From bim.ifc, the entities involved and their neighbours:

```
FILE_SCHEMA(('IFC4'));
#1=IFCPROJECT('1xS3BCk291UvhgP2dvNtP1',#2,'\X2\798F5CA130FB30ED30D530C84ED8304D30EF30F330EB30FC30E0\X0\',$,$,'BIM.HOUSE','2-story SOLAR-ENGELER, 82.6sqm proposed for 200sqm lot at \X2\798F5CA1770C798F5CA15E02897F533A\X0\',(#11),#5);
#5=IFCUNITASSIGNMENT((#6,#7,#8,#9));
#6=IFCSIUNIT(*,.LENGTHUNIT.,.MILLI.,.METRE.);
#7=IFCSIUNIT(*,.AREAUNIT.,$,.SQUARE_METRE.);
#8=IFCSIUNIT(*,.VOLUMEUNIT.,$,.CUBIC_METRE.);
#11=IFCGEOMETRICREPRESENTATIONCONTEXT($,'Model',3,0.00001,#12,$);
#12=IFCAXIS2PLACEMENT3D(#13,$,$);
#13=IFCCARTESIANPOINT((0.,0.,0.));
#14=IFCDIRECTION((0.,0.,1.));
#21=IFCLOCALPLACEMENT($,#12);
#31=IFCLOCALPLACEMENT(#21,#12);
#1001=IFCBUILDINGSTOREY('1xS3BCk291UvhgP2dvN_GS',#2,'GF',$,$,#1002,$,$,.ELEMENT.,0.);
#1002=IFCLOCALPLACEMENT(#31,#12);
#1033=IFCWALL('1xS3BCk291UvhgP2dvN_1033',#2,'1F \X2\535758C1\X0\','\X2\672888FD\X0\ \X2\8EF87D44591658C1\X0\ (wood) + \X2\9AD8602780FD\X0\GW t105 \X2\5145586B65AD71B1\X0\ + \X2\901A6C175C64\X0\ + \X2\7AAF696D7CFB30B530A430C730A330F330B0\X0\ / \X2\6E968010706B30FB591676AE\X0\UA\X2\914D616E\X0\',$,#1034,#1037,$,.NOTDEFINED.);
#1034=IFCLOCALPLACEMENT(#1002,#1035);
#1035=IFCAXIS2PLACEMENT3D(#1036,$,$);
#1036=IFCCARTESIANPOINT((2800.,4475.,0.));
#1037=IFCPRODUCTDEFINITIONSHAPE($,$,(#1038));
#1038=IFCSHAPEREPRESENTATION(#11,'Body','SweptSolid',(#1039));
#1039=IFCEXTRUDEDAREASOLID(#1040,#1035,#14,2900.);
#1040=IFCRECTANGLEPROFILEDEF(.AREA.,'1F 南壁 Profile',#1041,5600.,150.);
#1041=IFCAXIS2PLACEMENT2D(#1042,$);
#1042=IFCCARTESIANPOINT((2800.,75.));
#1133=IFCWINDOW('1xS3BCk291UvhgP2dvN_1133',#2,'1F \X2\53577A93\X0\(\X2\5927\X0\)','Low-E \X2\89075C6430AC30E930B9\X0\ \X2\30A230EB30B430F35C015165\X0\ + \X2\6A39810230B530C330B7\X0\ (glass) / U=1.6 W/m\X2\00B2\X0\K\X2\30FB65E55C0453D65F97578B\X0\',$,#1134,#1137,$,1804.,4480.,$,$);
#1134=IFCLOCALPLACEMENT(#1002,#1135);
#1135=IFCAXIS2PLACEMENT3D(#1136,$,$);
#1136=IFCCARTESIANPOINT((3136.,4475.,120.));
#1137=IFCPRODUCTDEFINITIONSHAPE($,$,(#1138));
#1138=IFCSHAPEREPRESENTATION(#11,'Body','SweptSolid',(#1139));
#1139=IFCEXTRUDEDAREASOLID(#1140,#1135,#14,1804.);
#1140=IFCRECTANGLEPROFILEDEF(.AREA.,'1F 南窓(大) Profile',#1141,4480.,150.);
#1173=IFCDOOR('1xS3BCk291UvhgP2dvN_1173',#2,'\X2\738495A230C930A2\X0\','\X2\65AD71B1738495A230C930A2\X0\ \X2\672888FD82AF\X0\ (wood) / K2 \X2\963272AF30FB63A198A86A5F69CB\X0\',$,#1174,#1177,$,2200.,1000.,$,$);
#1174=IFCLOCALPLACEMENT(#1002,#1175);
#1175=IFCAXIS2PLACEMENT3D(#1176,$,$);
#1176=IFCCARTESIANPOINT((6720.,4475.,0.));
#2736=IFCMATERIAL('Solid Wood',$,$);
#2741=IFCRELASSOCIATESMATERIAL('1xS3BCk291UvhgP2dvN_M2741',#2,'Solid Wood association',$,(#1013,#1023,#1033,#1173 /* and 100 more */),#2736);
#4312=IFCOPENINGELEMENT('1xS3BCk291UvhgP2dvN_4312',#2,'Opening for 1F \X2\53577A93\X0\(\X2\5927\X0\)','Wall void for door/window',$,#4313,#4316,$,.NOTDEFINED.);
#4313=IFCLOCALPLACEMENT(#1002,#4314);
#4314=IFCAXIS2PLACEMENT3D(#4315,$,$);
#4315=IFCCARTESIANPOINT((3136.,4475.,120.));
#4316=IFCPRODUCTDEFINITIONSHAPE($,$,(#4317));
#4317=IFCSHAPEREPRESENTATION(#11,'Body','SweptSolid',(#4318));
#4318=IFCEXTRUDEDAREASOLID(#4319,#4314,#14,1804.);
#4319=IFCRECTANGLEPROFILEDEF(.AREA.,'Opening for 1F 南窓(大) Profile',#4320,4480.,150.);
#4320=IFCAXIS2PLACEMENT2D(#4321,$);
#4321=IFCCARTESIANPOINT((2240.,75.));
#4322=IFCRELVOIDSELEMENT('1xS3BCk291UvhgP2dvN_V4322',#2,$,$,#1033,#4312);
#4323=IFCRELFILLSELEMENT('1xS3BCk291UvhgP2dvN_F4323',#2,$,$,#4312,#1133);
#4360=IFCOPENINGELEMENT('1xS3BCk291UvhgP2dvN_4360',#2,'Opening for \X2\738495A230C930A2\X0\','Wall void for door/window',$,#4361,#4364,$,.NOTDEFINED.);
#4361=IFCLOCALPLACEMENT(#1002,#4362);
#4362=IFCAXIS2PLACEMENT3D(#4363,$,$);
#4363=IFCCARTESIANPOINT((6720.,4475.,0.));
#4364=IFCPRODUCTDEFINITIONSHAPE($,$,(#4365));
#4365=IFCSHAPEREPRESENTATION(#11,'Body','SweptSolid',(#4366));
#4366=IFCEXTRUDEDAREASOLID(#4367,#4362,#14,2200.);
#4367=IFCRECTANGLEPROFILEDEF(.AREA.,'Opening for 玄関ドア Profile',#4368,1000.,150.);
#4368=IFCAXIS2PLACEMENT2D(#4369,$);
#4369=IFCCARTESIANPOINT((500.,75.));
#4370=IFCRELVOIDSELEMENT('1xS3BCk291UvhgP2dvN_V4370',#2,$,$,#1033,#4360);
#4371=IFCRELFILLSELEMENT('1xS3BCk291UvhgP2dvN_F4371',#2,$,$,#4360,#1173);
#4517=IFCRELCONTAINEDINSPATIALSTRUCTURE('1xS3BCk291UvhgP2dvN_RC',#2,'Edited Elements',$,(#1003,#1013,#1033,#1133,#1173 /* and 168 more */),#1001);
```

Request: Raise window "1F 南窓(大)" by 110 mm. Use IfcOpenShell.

```python
import numpy as np
import ifcopenshell
import ifcopenshell.api.geometry
import ifcopenshell.util.placement
import ifcopenshell.util.unit

model = ifcopenshell.open("bim.ifc")
unit_scale = ifcopenshell.util.unit.calculate_unit_scale(model)

window = model.by_guid("1xS3BCk291UvhgP2dvN_1133")
opening = window.FillsVoids[0].RelatingOpeningElement
dz = 0.11 / unit_scale

shift = np.array([0.0, 0.0, dz])
# The window is not placed relative to its opening, so move both.
for product in (opening, window):
    matrix = ifcopenshell.util.placement.get_local_placement(product.ObjectPlacement)
    matrix[:3, 3] += shift
    ifcopenshell.api.geometry.edit_object_placement(model, product=product, matrix=matrix, is_si=False)

print(f"moved by {dz * unit_scale:+.3f} m")

model.write("bim_v2.ifc")
```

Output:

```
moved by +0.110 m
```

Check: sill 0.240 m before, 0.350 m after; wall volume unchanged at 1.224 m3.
